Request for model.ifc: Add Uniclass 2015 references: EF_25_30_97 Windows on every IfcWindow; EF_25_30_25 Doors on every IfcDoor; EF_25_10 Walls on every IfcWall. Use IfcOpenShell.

First a look at what the model holds.

```python
import ifcopenshell

model = ifcopenshell.open("model.ifc")
print(model.schema)
print("classifications:", [c.Name for c in model.by_type("IfcClassification")])
for ifc_class in ("IfcDoor", "IfcRoof", "IfcStair", "IfcWall", "IfcWindow"):
    print(ifc_class, len(model.by_type(ifc_class)))
```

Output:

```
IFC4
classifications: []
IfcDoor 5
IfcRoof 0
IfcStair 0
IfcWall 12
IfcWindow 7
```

```python
import ifcopenshell
import ifcopenshell.api.classification

model = ifcopenshell.open("model.ifc")

system = ifcopenshell.api.classification.add_classification(model, classification="Uniclass 2015")

codes = {
    "IfcWindow": ("EF_25_30_97", "Windows"),
    "IfcDoor": ("EF_25_30_25", "Doors"),
    "IfcWall": ("EF_25_10", "Walls"),
}
for ifc_class, (code, name) in codes.items():
    products = model.by_type(ifc_class)
    ifcopenshell.api.classification.add_reference(
        model, products=products, classification=system, identification=code, name=name
    )
    print(code, len(products))

model.write("model_edited.ifc")
```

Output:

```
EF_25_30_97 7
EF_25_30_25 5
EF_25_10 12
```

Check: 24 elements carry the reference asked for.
